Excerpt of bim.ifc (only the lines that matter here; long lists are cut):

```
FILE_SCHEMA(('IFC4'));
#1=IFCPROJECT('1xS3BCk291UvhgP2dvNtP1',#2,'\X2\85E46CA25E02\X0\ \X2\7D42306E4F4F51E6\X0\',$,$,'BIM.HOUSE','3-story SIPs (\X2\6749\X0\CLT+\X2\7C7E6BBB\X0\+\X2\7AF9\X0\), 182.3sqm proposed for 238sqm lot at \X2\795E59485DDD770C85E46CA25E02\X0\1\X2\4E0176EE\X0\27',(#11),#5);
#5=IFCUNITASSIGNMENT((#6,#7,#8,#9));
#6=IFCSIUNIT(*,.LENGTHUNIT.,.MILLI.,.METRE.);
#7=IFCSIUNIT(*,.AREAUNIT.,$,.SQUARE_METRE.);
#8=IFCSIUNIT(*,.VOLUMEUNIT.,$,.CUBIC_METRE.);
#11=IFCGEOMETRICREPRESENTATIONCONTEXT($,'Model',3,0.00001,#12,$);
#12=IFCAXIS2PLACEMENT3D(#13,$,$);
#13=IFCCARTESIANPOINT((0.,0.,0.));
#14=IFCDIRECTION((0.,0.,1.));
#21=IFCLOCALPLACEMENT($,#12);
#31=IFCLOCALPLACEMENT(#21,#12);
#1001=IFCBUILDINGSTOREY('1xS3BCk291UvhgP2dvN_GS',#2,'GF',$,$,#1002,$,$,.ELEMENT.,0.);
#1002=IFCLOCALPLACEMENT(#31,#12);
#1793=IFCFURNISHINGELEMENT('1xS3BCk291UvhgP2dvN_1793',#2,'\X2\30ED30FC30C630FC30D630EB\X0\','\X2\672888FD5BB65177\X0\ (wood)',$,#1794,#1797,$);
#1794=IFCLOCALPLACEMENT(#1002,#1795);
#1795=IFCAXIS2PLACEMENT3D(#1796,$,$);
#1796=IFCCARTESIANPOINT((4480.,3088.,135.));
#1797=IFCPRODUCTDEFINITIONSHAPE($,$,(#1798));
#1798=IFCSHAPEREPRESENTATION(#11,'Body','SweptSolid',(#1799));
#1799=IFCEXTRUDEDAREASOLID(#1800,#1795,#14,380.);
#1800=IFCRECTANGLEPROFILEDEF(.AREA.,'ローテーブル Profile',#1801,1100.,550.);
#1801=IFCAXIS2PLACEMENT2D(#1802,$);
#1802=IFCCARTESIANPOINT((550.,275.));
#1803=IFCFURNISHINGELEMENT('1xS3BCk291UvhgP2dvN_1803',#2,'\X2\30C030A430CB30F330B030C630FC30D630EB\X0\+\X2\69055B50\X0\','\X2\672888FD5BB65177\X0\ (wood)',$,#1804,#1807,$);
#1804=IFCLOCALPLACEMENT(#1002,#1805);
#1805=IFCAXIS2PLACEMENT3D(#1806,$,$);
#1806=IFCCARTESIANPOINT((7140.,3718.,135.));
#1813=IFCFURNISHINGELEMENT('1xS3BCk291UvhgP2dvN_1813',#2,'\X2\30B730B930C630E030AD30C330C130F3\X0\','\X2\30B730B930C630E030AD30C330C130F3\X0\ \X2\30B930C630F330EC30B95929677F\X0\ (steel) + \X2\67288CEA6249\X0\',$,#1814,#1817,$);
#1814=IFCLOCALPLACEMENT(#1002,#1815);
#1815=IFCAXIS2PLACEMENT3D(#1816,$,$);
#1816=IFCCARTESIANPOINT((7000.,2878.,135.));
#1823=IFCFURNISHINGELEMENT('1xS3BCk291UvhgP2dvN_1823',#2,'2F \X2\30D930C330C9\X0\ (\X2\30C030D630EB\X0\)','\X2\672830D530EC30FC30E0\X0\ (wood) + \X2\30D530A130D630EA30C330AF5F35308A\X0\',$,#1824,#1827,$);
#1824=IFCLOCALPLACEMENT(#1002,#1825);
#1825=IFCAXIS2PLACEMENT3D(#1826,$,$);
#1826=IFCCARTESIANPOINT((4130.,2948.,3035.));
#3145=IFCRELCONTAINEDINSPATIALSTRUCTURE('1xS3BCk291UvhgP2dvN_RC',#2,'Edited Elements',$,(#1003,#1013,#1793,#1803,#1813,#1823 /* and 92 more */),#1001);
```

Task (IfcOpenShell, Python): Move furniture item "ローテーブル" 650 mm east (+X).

```python
import ifcopenshell
import ifcopenshell.api.geometry
import ifcopenshell.util.placement
import ifcopenshell.util.unit

model = ifcopenshell.open("bim.ifc")
unit_scale = ifcopenshell.util.unit.calculate_unit_scale(model)

item = model.by_guid("1xS3BCk291UvhgP2dvN_1793")
matrix = ifcopenshell.util.placement.get_local_placement(item.ObjectPlacement)
matrix[0, 3] += 0.65 / unit_scale
ifcopenshell.api.geometry.edit_object_placement(model, product=item, matrix=matrix, is_si=False)

print(ifcopenshell.util.placement.get_local_placement(item.ObjectPlacement).round(3) + 0.0)

model.write("bim_v2.ifc")
```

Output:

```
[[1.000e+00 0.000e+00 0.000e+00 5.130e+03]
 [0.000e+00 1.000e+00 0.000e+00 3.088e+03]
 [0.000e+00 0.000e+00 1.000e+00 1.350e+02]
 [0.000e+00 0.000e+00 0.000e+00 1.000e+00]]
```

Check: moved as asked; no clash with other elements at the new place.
